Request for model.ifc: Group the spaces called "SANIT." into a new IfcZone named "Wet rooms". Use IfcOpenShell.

First a look at what the model holds.

```python
import ifcopenshell

model = ifcopenshell.open("model.ifc")
print(model.schema)
seen = {}
for space in model.by_type("IfcSpace"):
    seen[space.LongName] = seen.get(space.LongName, 0) + 1
for name, count in sorted(seen.items(), key=str):
    print(count, "x", name)
print("zones:", [z.Name for z in model.by_type("IfcZone")][:20])
```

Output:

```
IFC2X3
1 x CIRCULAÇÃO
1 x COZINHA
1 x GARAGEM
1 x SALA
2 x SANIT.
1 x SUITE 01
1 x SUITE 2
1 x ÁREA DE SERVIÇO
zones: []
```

```python
import ifcopenshell
import ifcopenshell.api.group
import ifcopenshell.api.root

model = ifcopenshell.open("model.ifc")

names = {"SANIT."}
spaces = [s for s in model.by_type("IfcSpace") if s.LongName in names]

zone = ifcopenshell.api.root.create_entity(model, ifc_class="IfcZone", name="Wet rooms")
ifcopenshell.api.group.assign_group(model, products=spaces, group=zone)
print(len(spaces), "spaces in", zone.Name)

model.write("model-out.ifc")
```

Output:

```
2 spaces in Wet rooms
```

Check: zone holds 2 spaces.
